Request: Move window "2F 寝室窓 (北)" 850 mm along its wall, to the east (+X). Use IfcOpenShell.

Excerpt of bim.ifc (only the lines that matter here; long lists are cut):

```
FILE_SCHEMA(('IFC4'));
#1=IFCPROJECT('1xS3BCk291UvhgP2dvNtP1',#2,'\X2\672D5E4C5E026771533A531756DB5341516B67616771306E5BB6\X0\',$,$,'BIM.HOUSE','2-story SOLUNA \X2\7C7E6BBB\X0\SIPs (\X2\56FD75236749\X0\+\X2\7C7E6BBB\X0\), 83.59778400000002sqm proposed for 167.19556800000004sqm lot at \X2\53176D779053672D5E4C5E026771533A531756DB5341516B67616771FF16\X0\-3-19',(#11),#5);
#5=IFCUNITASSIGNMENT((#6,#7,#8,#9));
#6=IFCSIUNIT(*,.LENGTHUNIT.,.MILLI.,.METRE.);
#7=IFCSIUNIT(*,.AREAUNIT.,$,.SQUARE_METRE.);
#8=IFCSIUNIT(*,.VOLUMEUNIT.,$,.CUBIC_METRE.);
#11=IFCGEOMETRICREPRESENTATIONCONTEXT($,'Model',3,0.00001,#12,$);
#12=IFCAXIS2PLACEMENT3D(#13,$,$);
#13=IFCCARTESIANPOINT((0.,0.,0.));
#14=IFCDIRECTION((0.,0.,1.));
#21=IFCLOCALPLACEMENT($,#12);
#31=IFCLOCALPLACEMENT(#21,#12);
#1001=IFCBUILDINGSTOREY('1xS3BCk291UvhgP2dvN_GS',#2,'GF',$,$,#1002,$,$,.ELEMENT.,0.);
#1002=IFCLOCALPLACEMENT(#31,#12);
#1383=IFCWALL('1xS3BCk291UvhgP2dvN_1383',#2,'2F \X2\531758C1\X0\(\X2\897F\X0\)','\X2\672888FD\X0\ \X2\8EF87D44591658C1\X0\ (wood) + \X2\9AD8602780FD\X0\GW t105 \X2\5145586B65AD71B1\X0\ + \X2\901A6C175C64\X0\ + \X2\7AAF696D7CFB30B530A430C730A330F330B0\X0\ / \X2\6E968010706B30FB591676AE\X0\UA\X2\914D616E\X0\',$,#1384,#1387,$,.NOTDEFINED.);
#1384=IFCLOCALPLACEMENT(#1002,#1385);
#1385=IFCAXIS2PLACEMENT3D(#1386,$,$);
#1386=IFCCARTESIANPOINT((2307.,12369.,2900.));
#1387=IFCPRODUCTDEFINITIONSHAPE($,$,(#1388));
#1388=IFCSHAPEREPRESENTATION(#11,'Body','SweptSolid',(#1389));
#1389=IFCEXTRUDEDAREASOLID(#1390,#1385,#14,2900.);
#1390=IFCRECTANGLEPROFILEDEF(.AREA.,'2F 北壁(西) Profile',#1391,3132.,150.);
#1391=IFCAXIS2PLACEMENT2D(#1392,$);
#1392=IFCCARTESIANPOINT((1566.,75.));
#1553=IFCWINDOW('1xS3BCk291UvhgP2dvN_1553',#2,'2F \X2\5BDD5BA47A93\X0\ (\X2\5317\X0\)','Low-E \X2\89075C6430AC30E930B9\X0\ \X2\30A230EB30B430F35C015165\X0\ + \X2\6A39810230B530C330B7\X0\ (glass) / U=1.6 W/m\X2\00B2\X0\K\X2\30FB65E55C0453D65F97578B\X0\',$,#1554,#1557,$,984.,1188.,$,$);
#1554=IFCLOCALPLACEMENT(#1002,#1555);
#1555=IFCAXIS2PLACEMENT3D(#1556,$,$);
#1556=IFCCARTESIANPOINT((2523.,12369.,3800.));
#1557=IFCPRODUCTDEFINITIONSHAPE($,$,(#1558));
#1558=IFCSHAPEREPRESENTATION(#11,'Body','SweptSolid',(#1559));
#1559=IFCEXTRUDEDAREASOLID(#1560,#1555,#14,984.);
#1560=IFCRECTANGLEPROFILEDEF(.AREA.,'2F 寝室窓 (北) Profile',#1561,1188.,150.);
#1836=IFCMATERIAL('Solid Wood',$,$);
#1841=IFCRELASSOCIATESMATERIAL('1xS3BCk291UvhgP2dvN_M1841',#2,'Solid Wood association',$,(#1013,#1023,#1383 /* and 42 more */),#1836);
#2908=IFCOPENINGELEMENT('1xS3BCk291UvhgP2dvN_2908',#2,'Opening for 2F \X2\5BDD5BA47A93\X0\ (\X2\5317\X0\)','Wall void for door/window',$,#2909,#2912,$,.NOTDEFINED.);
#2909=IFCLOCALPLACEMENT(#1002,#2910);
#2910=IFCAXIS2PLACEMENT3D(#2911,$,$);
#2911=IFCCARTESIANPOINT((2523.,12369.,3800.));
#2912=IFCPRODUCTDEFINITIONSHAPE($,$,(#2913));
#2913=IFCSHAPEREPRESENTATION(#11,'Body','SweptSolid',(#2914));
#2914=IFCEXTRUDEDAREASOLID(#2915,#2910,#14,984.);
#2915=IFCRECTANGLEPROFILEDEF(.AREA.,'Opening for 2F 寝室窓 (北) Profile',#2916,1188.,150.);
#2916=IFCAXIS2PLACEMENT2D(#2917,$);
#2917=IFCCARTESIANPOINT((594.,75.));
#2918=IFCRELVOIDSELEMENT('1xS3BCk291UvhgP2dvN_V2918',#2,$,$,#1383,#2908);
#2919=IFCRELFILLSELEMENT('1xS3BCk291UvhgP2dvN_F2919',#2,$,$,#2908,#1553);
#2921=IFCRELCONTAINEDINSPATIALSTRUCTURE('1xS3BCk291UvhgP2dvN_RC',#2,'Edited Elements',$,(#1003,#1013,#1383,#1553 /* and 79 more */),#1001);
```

```python
import ifcopenshell
import ifcopenshell.api.geometry
import ifcopenshell.util.placement
import ifcopenshell.util.unit

model = ifcopenshell.open("bim.ifc")
unit_scale = ifcopenshell.util.unit.calculate_unit_scale(model)

window = model.by_id(1553)
opening = window.FillsVoids[0].RelatingOpeningElement
wall = opening.VoidsElements[0].RelatingBuildingElement

wall_matrix = ifcopenshell.util.placement.get_local_placement(wall.ObjectPlacement)
shift = wall_matrix[:3, 0] * 0.85 / unit_scale
before = ifcopenshell.util.placement.get_local_placement(window.ObjectPlacement)[:3, 3].copy()

# The window is not placed relative to its opening, so move both.
for product in (opening, window):
    matrix = ifcopenshell.util.placement.get_local_placement(product.ObjectPlacement)
    matrix[:3, 3] += shift
    ifcopenshell.api.geometry.edit_object_placement(model, product=product, matrix=matrix, is_si=False)

after = ifcopenshell.util.placement.get_local_placement(window.ObjectPlacement)[:3, 3]
print("window moved by", (after - before).round(3) + 0.0)

model.write("bim_updated.ifc")
```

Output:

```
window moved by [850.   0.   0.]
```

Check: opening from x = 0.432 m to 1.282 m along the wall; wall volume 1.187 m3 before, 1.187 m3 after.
